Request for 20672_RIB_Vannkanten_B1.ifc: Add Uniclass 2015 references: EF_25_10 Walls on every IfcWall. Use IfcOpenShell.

First a look at what the model holds.

```python
import ifcopenshell

model = ifcopenshell.open("20672_RIB_Vannkanten_B1.ifc")
print(model.schema)
print("classifications:", [c.Name for c in model.by_type("IfcClassification")])
for ifc_class in ("IfcDoor", "IfcRoof", "IfcStair", "IfcWall", "IfcWindow"):
    print(ifc_class, len(model.by_type(ifc_class)))
```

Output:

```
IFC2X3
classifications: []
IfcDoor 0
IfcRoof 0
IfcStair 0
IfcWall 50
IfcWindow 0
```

```python
import ifcopenshell
import ifcopenshell.api.classification

model = ifcopenshell.open("20672_RIB_Vannkanten_B1.ifc")

# IFC2X3 requires Source and Edition and has no link from the project to the system.
system = model.create_entity("IfcClassification", Source="NBS", Edition="2015", Name="Uniclass 2015")

codes = {
    "IfcWall": ("EF_25_10", "Walls"),
}
for ifc_class, (code, name) in codes.items():
    products = model.by_type(ifc_class)
    ifcopenshell.api.classification.add_reference(
        model, products=products, classification=system, identification=code, name=name
    )
    print(code, len(products))

model.write("20672_RIB_Vannkanten_B1_rev.ifc")
```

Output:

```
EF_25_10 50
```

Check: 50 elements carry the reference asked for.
